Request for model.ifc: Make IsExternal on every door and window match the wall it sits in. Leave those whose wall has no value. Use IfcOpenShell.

First a look at what the model holds.

```python
import ifcopenshell
import ifcopenshell.util.element

model = ifcopenshell.open("model.ifc")
print(model.schema)
seen = {}
for e in model.by_type("IfcDoor") + model.by_type("IfcWindow"):
    if not e.FillsVoids:
        continue
    host = e.FillsVoids[0].RelatingOpeningElement.VoidsElements[0].RelatingBuildingElement
    own = ifcopenshell.util.element.get_pset(e, f"Pset_{e.is_a()[3:].removesuffix('StandardCase')}Common", "IsExternal")
    wall = ifcopenshell.util.element.get_pset(host, "Pset_WallCommon", "IsExternal")
    seen[e.is_a(), own, wall] = seen.get((e.is_a(), own, wall), 0) + 1
for (cls, own, wall), count in sorted(seen.items(), key=str):
    print(count, cls, "IsExternal:", own, "| host wall:", wall)
```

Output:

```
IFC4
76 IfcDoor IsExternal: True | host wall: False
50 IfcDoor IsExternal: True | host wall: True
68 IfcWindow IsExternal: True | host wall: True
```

```python
import ifcopenshell
import ifcopenshell.api.pset
import ifcopenshell.util.element

model = ifcopenshell.open("model.ifc")

count = 0
for ifc_class, pset_name in (("IfcDoor", "Pset_DoorCommon"), ("IfcWindow", "Pset_WindowCommon")):
    for e in model.by_type(ifc_class):
        if not e.FillsVoids:
            continue
        host = e.FillsVoids[0].RelatingOpeningElement.VoidsElements[0].RelatingBuildingElement
        external = ifcopenshell.util.element.get_pset(host, "Pset_WallCommon", "IsExternal")
        if external is None or ifcopenshell.util.element.get_pset(e, pset_name, "IsExternal") == external:
            continue
        pset = ifcopenshell.api.pset.add_pset(model, product=e, name=pset_name)
        ifcopenshell.api.pset.edit_pset(model, pset=pset, properties={"IsExternal": external})
        count += 1

print(count, "updated")

model.write("model_updated.ifc")
```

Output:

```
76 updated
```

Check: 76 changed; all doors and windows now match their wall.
